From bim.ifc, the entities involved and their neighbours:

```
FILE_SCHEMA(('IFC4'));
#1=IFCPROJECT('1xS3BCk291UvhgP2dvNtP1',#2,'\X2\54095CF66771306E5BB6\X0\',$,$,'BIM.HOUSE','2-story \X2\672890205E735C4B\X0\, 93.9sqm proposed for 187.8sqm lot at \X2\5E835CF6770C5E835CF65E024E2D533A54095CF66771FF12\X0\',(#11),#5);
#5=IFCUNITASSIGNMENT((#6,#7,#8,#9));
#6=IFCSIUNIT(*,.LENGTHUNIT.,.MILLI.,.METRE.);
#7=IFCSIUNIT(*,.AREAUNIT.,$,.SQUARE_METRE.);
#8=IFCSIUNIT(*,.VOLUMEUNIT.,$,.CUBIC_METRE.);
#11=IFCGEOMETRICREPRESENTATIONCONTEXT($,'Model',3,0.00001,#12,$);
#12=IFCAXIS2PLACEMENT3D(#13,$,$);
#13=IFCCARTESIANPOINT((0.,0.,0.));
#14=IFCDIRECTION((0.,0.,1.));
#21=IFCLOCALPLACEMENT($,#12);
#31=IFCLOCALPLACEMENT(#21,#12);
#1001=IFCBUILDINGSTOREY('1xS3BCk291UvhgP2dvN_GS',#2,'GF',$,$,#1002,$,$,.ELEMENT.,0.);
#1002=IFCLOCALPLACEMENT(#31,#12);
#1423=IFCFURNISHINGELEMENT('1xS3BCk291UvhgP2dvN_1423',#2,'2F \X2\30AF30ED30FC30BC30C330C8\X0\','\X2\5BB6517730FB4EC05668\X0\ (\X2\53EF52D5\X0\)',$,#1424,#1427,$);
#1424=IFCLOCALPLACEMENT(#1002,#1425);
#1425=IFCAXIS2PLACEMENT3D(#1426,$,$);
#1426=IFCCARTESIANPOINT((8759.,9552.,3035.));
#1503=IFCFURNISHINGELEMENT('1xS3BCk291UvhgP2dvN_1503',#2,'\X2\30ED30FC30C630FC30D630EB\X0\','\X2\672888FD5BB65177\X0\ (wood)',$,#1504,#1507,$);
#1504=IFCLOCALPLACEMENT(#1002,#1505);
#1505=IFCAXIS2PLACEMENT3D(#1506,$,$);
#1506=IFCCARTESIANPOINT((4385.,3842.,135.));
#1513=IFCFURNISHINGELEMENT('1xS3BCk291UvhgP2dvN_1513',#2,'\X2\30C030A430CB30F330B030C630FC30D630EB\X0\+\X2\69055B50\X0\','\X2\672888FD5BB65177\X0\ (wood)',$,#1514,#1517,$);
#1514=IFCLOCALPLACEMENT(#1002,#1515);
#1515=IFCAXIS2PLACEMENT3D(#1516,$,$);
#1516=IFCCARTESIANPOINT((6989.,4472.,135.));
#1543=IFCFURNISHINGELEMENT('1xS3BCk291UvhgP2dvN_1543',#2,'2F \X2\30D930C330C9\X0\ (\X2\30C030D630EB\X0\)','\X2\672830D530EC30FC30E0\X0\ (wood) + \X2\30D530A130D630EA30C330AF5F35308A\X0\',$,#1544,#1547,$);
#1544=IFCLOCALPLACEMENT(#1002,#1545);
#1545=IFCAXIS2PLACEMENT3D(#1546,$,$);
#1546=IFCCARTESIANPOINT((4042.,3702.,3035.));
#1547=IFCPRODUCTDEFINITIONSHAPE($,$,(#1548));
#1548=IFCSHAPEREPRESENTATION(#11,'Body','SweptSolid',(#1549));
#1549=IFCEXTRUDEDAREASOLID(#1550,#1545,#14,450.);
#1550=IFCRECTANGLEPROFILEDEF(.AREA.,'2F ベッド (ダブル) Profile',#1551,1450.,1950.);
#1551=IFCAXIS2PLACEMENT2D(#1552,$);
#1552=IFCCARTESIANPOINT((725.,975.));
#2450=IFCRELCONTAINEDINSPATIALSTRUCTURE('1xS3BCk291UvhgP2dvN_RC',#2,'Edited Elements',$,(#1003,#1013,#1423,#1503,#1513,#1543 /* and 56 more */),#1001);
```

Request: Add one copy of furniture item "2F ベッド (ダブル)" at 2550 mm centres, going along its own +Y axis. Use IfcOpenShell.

```python
import ifcopenshell
import ifcopenshell.api.geometry
import ifcopenshell.api.root
import ifcopenshell.util.element
import ifcopenshell.util.placement
import ifcopenshell.util.unit

model = ifcopenshell.open("bim.ifc")
unit_scale = ifcopenshell.util.unit.calculate_unit_scale(model)


def reuse_history(source, copy):
    """copy_class also copies each property set's owner history, people and application; keep the originals."""
    for rel in copy.IsDefinedBy:
        if rel.is_a("IfcRelDefinesByProperties") and (history := rel.RelatingPropertyDefinition.OwnerHistory):
            rel.RelatingPropertyDefinition.OwnerHistory = source.OwnerHistory
            ifcopenshell.util.element.remove_deep2(model, history)


source = model.by_guid("1xS3BCk291UvhgP2dvN_1543")
base = ifcopenshell.util.placement.get_local_placement(source.ObjectPlacement)
step = base[:3, 1] * 2.55 / unit_scale

for i in range(1, 2):
    copy = ifcopenshell.api.root.copy_class(model, product=source)
    copy.Representation = ifcopenshell.util.element.copy_deep(
        model, source.Representation, exclude=["IfcGeometricRepresentationContext", "IfcRepresentationMap"]
    )
    reuse_history(source, copy)
    matrix = base.copy()
    matrix[:3, 3] += i * step
    print("added at", matrix[:3, 3].round(3) + 0.0)
    ifcopenshell.api.geometry.edit_object_placement(model, product=copy, matrix=matrix, is_si=False)

model.write("bim_rev.ifc")
```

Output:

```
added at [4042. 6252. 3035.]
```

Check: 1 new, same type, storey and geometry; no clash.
